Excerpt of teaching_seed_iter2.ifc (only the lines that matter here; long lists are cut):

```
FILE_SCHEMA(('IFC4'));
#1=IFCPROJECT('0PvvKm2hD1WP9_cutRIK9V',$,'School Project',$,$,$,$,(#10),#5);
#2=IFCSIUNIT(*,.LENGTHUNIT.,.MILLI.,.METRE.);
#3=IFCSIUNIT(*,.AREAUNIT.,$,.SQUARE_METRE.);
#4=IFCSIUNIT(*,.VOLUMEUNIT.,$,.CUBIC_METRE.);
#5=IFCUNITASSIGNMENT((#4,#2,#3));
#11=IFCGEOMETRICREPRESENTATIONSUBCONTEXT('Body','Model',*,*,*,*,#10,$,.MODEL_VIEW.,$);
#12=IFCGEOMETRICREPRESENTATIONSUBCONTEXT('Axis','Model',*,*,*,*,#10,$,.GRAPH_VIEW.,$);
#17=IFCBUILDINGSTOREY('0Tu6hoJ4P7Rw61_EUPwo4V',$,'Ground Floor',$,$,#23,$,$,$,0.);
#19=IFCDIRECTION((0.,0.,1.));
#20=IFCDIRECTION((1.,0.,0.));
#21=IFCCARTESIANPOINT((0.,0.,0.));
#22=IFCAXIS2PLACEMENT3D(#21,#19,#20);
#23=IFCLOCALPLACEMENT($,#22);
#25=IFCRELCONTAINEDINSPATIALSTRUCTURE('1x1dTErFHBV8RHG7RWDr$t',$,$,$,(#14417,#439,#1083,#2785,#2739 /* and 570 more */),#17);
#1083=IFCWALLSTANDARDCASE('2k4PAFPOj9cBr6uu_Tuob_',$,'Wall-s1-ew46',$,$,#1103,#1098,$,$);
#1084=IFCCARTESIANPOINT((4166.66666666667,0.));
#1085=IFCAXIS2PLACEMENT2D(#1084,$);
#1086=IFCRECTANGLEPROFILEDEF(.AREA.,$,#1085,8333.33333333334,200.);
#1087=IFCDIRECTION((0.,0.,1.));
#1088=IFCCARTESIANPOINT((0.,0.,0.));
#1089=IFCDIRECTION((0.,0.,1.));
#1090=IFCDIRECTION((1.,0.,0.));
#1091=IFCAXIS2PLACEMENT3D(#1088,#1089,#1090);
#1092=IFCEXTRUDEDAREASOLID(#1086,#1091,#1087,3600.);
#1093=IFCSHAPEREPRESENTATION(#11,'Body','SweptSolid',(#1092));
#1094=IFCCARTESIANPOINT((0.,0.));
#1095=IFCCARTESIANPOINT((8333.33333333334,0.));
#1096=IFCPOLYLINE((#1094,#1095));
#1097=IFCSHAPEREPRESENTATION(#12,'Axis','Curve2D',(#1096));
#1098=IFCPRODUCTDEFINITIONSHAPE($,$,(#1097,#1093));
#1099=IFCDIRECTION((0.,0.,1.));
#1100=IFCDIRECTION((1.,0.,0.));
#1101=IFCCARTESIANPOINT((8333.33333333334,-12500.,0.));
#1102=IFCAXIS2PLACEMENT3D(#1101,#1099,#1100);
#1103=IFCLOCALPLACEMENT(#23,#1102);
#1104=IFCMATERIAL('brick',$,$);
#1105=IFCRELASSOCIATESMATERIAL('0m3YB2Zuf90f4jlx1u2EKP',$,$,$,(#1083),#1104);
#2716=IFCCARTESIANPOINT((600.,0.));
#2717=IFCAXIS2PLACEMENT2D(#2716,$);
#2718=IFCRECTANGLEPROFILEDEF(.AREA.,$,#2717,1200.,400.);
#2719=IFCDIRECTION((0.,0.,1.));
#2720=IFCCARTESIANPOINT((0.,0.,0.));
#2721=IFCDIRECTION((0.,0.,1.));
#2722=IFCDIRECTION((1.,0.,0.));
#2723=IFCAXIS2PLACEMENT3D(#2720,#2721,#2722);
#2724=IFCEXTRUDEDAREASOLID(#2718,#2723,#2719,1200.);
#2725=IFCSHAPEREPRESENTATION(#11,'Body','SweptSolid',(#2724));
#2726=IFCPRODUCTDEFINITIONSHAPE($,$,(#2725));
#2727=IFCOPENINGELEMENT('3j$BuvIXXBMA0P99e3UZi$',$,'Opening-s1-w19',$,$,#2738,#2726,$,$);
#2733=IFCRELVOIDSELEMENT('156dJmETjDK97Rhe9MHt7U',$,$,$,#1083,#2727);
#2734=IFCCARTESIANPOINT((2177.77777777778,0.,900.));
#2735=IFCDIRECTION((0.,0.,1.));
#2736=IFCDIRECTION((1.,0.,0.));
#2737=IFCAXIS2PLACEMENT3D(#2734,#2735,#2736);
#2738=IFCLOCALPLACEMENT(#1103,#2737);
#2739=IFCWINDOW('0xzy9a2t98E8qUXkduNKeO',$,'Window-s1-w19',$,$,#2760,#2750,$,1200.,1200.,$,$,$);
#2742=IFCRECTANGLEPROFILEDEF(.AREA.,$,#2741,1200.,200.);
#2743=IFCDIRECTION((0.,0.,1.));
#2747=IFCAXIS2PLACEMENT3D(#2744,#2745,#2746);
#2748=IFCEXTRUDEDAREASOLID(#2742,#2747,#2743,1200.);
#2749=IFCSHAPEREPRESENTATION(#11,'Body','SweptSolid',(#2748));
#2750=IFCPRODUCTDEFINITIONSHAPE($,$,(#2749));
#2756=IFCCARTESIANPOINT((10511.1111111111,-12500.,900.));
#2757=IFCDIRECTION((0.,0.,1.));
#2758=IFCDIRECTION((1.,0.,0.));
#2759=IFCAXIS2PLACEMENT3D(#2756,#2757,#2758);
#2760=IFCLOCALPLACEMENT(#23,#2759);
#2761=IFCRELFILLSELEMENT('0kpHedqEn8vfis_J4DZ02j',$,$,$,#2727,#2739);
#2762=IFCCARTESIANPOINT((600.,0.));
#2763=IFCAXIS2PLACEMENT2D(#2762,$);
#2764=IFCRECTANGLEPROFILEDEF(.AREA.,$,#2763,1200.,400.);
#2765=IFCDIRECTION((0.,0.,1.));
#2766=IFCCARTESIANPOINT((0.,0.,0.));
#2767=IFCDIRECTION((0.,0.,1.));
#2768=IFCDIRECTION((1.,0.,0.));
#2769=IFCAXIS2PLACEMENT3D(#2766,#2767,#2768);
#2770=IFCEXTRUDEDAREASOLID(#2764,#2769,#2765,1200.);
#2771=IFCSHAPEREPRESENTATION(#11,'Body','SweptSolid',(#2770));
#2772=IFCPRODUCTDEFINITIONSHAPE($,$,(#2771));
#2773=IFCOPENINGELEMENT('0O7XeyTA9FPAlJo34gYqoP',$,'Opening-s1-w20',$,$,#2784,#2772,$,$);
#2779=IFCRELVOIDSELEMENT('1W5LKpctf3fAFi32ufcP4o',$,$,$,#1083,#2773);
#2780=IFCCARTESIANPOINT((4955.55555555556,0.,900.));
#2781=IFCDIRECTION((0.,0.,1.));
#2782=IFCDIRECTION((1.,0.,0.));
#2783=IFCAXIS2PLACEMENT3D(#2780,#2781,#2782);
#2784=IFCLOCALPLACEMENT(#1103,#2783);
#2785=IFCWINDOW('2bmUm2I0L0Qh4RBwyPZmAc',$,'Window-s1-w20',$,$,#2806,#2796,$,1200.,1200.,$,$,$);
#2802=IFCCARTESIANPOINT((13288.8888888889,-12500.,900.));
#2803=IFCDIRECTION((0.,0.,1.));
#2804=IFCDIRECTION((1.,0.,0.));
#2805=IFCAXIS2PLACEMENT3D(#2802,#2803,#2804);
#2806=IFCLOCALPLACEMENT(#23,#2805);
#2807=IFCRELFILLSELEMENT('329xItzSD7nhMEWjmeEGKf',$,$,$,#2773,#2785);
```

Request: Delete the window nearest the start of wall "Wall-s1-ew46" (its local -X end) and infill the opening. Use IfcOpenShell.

```python
import ifcopenshell
import ifcopenshell.api.feature
import ifcopenshell.api.root
import ifcopenshell.geom
import ifcopenshell.util.shape

model = ifcopenshell.open("teaching_seed_iter2.ifc")
settings = ifcopenshell.geom.settings()


def volume(element):
    """Net volume in cubic metres, openings subtracted."""
    shape = ifcopenshell.geom.create_shape(settings, element)
    return ifcopenshell.util.shape.get_volume(shape.geometry)


window = model.by_guid("0xzy9a2t98E8qUXkduNKeO")
opening = window.FillsVoids[0].RelatingOpeningElement
wall = opening.VoidsElements[0].RelatingBuildingElement
before = volume(wall)

ifcopenshell.api.root.remove_product(model, product=window)
ifcopenshell.api.feature.remove_feature(model, feature=opening)

after = volume(wall)

print(f"wall volume {before:.3f} -> {after:.3f} m3")

model.write("teaching_seed_iter2-out.ifc")
```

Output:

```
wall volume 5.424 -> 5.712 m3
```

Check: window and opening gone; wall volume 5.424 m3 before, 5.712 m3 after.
